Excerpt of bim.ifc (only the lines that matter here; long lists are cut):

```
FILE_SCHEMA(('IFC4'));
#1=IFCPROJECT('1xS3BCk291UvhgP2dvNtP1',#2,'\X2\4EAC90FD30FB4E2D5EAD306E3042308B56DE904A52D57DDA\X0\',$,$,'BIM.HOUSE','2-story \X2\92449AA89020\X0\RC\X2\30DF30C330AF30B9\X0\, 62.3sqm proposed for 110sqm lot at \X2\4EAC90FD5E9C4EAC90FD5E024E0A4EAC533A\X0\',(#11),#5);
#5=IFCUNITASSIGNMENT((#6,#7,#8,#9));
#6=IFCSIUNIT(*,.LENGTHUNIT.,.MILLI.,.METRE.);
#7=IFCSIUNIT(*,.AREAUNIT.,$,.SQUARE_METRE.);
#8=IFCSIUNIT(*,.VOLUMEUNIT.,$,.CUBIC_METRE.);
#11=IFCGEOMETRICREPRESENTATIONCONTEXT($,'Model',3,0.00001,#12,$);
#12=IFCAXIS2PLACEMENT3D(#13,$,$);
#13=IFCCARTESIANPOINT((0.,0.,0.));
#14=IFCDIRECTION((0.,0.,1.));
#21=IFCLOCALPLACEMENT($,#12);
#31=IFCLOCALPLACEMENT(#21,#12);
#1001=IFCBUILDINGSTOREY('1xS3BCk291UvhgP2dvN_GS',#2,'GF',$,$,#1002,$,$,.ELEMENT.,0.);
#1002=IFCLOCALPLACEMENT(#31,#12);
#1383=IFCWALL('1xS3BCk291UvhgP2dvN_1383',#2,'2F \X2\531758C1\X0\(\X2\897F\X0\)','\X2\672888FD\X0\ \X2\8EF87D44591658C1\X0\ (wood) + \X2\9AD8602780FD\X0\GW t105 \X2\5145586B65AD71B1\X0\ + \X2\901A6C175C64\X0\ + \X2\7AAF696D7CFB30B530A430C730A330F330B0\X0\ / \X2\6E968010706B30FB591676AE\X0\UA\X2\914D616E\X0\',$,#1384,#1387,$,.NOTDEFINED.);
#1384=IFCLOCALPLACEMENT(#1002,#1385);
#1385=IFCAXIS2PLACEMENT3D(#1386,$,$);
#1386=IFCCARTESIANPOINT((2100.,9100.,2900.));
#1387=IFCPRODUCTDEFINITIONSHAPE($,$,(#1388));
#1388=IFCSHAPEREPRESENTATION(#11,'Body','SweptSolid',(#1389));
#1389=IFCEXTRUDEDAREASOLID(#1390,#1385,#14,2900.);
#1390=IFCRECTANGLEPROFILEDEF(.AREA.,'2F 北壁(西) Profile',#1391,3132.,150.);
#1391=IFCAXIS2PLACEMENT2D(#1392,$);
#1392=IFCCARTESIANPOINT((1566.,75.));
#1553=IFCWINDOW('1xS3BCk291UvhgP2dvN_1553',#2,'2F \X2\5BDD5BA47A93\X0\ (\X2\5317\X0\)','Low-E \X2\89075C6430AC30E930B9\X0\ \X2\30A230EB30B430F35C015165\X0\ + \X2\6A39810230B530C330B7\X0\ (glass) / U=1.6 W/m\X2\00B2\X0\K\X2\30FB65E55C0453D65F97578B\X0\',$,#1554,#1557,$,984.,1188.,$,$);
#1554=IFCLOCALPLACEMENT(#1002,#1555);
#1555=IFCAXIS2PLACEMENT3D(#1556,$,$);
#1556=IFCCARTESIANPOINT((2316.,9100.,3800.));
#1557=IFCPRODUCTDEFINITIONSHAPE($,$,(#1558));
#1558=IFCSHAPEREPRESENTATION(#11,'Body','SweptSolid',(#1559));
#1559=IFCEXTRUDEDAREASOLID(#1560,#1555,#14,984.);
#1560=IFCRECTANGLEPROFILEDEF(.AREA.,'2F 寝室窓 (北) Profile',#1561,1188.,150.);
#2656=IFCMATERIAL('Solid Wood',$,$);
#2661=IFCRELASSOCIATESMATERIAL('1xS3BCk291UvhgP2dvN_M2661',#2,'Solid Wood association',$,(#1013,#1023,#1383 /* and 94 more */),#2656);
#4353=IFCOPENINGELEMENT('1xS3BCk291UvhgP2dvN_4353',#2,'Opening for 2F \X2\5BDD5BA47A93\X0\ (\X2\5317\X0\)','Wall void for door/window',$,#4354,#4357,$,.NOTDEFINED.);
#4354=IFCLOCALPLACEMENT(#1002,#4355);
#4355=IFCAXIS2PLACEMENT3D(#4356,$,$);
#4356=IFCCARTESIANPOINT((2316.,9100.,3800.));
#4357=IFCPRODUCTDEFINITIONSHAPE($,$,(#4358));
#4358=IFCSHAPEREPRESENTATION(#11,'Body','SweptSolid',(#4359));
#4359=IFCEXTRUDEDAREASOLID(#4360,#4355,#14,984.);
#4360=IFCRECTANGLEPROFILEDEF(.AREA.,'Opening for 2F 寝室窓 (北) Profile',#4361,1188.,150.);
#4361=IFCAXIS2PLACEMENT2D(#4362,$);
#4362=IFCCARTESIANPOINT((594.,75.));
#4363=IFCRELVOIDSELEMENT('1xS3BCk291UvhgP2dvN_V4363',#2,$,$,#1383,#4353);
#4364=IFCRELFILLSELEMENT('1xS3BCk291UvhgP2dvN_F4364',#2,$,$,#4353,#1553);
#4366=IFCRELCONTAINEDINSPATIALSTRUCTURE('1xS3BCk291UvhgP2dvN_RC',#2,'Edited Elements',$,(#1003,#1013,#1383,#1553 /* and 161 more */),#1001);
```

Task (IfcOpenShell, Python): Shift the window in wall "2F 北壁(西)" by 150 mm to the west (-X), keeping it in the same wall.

```python
import ifcopenshell
import ifcopenshell.api.geometry
import ifcopenshell.util.placement
import ifcopenshell.util.unit

model = ifcopenshell.open("bim.ifc")
unit_scale = ifcopenshell.util.unit.calculate_unit_scale(model)

window = model.by_id(1553)
opening = window.FillsVoids[0].RelatingOpeningElement
wall = opening.VoidsElements[0].RelatingBuildingElement

wall_matrix = ifcopenshell.util.placement.get_local_placement(wall.ObjectPlacement)
shift = wall_matrix[:3, 0] * -0.15 / unit_scale
before = ifcopenshell.util.placement.get_local_placement(window.ObjectPlacement)[:3, 3].copy()

# The window is not placed relative to its opening, so move both.
for product in (opening, window):
    matrix = ifcopenshell.util.placement.get_local_placement(product.ObjectPlacement)
    matrix[:3, 3] += shift
    ifcopenshell.api.geometry.edit_object_placement(model, product=product, matrix=matrix, is_si=False)

after = ifcopenshell.util.placement.get_local_placement(window.ObjectPlacement)[:3, 3]
print("window moved by", (after - before).round(3) + 0.0)

model.write("bim_edited.ifc")
```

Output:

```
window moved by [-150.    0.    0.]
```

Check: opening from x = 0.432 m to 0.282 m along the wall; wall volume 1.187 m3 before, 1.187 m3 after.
